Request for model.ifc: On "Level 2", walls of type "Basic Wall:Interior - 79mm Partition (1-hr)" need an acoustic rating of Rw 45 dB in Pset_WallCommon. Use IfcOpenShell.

First a look at what the model holds.

```python
import ifcopenshell
import ifcopenshell.util.element

model = ifcopenshell.open("model.ifc")
print(model.schema)
storey = next(s for s in model.by_type("IfcBuildingStorey") if s.Name == "Level 2")
walls = [e for e in ifcopenshell.util.element.get_decomposition(storey) if e.is_a("IfcWall")]
seen = {}
for e in walls:
    element_type = ifcopenshell.util.element.get_type(e)
    key = (element_type.Name if element_type != e and element_type else None, ifcopenshell.util.element.get_pset(e, "Pset_WallCommon", "AcousticRating"))
    seen[key] = seen.get(key, 0) + 1
for (name, value), count in sorted(seen.items(), key=str):
    print(count, "x", name, "|", value)
```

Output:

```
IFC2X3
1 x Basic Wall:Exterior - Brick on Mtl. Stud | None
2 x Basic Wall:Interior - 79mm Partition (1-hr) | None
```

```python
import ifcopenshell
import ifcopenshell.api.pset
import ifcopenshell.util.element

model = ifcopenshell.open("model.ifc")

storey = next(s for s in model.by_type("IfcBuildingStorey") if s.Name == "Level 2")
walls = [e for e in ifcopenshell.util.element.get_decomposition(storey) if e.is_a("IfcWall")]

count = 0
for e in walls:
    element_type = ifcopenshell.util.element.get_type(e)
    if element_type in (None, e) or element_type.Name != "Basic Wall:Interior - 79mm Partition (1-hr)":
        continue
    # add_pset returns the element's existing set when there is one.
    pset = ifcopenshell.api.pset.add_pset(model, product=e, name="Pset_WallCommon")
    ifcopenshell.api.pset.edit_pset(model, pset=pset, properties={"AcousticRating": "Rw 45 dB"})
    count += 1

print(count, "walls updated")

model.write("model_updated.ifc")
```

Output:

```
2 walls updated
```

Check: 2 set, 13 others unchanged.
